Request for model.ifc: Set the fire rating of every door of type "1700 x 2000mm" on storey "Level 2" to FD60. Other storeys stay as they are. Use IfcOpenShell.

First a look at what the model holds.

```python
import ifcopenshell
import ifcopenshell.util.element

model = ifcopenshell.open("model.ifc")
print(model.schema)
storey = next(s for s in model.by_type("IfcBuildingStorey") if s.Name == "Level 2")
doors = [e for e in ifcopenshell.util.element.get_decomposition(storey) if e.is_a("IfcDoor")]
seen = {}
for e in doors:
    element_type = ifcopenshell.util.element.get_type(e)
    key = (element_type.Name if element_type != e and element_type else None, ifcopenshell.util.element.get_pset(e, "Pset_DoorCommon", "FireRating"))
    seen[key] = seen.get(key, 0) + 1
for (name, value), count in sorted(seen.items(), key=str):
    print(count, "x", name, "|", value)
```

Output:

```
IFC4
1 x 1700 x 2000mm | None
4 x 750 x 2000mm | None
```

```python
import ifcopenshell
import ifcopenshell.api.pset
import ifcopenshell.util.element

model = ifcopenshell.open("model.ifc")

storey = next(s for s in model.by_type("IfcBuildingStorey") if s.Name == "Level 2")
doors = [e for e in ifcopenshell.util.element.get_decomposition(storey) if e.is_a("IfcDoor")]

count = 0
for e in doors:
    element_type = ifcopenshell.util.element.get_type(e)
    if element_type in (None, e) or element_type.Name != "1700 x 2000mm":
        continue
    # add_pset returns the element's existing set when there is one.
    pset = ifcopenshell.api.pset.add_pset(model, product=e, name="Pset_DoorCommon")
    ifcopenshell.api.pset.edit_pset(model, pset=pset, properties={"FireRating": "FD60"})
    count += 1

print(count, "doors updated")

model.write("model_updated.ifc")
```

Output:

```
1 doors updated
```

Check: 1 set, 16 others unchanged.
